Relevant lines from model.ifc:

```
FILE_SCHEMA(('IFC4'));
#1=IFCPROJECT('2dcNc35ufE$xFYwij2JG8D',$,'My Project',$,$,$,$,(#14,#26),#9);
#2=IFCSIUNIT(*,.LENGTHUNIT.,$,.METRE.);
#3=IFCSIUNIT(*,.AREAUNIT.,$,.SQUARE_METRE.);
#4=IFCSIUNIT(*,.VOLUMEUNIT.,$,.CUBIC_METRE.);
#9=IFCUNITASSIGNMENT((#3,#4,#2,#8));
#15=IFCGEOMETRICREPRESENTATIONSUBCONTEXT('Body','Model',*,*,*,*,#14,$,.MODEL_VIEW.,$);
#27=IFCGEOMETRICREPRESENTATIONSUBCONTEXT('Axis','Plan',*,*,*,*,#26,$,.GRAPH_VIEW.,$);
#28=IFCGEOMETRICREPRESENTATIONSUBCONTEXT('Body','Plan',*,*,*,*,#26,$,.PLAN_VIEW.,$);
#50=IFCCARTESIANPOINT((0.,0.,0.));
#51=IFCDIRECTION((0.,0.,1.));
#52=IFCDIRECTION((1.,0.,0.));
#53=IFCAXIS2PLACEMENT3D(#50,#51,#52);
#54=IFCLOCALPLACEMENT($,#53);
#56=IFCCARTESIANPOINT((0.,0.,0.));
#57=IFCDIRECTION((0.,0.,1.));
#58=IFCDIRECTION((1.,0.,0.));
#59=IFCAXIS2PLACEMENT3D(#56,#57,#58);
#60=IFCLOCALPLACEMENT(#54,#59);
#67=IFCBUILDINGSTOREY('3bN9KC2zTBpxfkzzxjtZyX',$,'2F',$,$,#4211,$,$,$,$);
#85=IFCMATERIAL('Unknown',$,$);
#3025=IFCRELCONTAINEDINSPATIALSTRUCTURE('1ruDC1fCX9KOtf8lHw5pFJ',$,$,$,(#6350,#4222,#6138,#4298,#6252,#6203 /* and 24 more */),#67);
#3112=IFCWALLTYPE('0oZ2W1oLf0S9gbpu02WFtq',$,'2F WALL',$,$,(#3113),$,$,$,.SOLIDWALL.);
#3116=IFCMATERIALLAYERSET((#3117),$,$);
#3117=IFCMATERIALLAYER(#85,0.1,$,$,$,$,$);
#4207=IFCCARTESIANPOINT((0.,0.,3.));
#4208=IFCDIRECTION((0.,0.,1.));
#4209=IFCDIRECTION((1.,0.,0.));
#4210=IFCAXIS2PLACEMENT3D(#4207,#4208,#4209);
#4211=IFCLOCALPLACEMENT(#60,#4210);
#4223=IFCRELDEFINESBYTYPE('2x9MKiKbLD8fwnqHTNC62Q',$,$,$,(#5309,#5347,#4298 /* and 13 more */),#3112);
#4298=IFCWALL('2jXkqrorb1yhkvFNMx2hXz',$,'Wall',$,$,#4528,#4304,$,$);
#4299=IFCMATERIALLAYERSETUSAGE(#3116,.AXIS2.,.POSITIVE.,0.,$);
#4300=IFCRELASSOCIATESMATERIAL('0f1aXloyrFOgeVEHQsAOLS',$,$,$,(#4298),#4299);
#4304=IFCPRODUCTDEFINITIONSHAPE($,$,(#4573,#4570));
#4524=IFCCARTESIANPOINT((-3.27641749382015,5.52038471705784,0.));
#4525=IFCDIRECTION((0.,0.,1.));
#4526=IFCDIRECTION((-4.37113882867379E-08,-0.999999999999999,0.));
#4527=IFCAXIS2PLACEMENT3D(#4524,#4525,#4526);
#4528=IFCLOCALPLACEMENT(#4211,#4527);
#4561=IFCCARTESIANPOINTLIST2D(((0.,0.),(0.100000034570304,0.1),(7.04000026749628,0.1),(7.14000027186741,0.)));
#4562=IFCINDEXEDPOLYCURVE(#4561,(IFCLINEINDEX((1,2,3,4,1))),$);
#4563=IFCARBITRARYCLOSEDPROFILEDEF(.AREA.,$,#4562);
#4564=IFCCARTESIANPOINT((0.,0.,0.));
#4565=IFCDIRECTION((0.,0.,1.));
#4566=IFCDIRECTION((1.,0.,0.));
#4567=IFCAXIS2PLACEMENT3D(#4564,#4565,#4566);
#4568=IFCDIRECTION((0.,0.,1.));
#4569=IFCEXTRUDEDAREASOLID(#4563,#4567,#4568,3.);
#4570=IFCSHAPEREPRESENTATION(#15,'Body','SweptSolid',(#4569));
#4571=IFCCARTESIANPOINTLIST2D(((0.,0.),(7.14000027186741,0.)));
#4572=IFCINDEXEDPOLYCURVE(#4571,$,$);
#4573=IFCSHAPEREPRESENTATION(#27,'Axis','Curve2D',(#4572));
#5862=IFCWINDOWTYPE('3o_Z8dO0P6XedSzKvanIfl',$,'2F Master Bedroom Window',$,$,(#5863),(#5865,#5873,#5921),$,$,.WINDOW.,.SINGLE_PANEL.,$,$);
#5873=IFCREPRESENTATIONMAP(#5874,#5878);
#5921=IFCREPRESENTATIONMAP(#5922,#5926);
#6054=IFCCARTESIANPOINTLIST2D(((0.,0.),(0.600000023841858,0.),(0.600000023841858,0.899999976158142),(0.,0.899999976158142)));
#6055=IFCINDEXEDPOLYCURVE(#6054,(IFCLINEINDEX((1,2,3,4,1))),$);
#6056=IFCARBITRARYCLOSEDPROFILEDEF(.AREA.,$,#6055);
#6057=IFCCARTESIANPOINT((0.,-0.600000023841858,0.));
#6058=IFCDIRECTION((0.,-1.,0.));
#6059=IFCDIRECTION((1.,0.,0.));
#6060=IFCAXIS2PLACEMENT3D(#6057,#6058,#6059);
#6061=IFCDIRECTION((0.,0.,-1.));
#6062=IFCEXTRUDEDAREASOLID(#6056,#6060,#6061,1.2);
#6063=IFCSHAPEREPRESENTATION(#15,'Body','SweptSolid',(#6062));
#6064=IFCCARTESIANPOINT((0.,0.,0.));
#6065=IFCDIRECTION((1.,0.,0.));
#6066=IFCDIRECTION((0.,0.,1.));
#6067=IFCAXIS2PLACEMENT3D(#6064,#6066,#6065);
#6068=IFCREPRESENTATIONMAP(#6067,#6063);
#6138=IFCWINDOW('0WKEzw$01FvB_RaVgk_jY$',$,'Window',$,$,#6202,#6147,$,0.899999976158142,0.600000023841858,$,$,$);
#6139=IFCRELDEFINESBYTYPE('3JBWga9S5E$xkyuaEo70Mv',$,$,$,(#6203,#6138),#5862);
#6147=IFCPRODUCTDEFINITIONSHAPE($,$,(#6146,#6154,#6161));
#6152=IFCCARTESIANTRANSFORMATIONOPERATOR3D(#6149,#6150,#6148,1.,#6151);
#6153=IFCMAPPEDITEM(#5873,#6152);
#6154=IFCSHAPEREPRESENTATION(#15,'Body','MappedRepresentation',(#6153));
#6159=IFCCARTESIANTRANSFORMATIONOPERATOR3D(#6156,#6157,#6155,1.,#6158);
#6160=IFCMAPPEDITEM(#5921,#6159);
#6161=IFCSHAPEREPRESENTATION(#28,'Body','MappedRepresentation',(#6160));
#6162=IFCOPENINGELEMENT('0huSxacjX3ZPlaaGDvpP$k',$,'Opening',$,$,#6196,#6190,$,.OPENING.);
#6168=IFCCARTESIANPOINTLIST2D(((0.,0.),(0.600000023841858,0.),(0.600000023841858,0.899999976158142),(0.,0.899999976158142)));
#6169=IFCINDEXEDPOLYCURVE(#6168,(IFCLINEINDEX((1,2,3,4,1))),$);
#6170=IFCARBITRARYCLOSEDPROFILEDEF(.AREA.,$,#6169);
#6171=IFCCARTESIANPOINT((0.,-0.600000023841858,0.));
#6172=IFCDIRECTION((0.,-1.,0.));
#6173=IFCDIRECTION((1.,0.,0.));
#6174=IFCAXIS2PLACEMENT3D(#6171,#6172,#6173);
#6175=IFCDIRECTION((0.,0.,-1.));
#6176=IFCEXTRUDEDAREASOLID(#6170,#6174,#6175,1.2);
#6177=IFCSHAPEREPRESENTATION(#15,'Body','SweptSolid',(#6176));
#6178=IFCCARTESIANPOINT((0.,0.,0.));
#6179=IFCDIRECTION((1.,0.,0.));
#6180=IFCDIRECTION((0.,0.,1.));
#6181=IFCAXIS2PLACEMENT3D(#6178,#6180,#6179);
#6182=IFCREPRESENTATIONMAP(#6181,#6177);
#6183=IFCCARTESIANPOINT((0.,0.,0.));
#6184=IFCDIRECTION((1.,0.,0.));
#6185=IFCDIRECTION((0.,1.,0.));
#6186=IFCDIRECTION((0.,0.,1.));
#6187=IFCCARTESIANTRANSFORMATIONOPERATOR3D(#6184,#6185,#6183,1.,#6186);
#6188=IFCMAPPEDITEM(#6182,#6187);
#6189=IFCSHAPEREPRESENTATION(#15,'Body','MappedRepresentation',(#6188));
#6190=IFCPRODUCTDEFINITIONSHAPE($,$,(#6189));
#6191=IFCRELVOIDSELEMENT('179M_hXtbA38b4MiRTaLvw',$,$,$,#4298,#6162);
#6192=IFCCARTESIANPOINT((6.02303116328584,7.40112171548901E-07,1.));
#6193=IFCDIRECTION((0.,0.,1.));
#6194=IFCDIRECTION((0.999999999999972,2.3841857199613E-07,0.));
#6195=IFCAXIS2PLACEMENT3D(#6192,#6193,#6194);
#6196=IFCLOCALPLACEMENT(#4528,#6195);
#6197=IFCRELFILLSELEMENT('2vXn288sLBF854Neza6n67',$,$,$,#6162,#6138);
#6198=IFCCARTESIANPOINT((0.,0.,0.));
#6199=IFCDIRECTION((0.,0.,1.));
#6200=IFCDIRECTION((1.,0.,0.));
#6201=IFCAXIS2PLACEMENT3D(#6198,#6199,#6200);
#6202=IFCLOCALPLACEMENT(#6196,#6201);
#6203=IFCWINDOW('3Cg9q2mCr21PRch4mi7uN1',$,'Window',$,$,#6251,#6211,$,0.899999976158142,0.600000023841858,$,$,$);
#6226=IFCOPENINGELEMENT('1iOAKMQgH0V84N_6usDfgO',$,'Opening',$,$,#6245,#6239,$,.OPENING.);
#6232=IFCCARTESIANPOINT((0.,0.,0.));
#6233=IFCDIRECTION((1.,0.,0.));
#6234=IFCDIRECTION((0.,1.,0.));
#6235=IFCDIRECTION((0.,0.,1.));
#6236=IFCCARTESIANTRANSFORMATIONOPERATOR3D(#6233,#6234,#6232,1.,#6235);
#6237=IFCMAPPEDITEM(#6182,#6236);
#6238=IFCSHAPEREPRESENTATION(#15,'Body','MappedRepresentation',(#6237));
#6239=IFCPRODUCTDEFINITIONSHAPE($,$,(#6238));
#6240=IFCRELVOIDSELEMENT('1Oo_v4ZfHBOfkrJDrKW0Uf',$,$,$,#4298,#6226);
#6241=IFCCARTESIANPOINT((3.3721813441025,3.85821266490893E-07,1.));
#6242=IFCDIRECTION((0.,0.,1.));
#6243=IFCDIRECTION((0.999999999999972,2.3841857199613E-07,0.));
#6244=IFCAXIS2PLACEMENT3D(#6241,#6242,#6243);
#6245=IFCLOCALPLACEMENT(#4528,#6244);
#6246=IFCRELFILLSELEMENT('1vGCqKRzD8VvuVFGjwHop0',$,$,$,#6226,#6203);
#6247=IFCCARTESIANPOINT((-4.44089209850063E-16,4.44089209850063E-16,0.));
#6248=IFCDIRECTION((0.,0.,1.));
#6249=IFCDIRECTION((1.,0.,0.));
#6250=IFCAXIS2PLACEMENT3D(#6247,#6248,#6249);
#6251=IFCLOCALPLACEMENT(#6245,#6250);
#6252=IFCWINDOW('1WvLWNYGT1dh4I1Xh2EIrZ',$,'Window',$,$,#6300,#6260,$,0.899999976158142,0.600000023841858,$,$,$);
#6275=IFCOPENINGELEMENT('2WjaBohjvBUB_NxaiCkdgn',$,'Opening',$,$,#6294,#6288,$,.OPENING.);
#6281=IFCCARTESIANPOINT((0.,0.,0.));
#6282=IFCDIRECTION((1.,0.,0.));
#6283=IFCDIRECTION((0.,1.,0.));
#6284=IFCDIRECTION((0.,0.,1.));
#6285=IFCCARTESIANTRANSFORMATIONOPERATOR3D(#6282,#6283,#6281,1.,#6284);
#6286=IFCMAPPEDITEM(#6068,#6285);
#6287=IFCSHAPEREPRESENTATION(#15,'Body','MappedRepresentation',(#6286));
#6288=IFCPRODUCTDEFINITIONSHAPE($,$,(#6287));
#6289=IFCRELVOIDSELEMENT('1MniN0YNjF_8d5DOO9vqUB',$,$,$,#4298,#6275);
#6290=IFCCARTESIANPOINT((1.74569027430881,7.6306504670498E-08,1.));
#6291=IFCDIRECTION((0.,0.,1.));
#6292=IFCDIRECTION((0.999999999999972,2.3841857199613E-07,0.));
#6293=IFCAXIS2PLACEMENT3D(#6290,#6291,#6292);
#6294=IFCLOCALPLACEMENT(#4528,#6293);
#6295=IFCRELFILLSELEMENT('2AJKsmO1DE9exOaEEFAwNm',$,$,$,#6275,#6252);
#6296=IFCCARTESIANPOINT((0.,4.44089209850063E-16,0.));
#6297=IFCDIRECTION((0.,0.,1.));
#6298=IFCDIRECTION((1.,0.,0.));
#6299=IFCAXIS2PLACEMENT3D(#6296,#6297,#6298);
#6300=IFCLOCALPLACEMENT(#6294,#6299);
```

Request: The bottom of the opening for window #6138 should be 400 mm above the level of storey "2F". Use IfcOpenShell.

```python
import numpy as np
import ifcopenshell
import ifcopenshell.api.geometry
import ifcopenshell.geom
import ifcopenshell.util.element
import ifcopenshell.util.placement
import ifcopenshell.util.shape
import ifcopenshell.util.unit

model = ifcopenshell.open("model.ifc")
unit_scale = ifcopenshell.util.unit.calculate_unit_scale(model)

window = model.by_guid("0WKEzw$01FvB_RaVgk_jY$")
opening = window.FillsVoids[0].RelatingOpeningElement
storey = ifcopenshell.util.element.get_container(window, ifc_class="IfcBuildingStorey")
level = ifcopenshell.util.placement.get_local_placement(storey.ObjectPlacement)[2, 3]

# The opening's origin need not be at the sill, so measure its lowest point.
shape = ifcopenshell.geom.create_shape(ifcopenshell.geom.settings(), opening)
bottom = ifcopenshell.util.shape.get_shape_bottom_elevation(shape, shape.geometry) / unit_scale
dz = level + 0.4 / unit_scale - bottom

shift = np.array([0.0, 0.0, dz])
# The window is placed relative to its opening, so it follows when the opening moves.
matrix = ifcopenshell.util.placement.get_local_placement(opening.ObjectPlacement)
matrix[:3, 3] += shift
ifcopenshell.api.geometry.edit_object_placement(
    model, product=opening, matrix=matrix, is_si=False, should_transform_children=True
)

print(f"moved by {dz * unit_scale:+.3f} m")

model.write("model-out.ifc")
```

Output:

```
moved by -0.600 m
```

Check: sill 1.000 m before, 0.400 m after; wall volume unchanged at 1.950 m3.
